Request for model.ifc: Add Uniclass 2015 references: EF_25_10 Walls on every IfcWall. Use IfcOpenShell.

First a look at what the model holds.

```python
import ifcopenshell

model = ifcopenshell.open("model.ifc")
print(model.schema)
print("classifications:", [c.Name for c in model.by_type("IfcClassification")])
for ifc_class in ("IfcDoor", "IfcRoof", "IfcStair", "IfcWall", "IfcWindow"):
    print(ifc_class, len(model.by_type(ifc_class)))
```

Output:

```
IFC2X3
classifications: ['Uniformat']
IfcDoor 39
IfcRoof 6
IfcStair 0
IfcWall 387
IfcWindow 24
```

```python
import ifcopenshell
import ifcopenshell.api.classification

model = ifcopenshell.open("model.ifc")

# IFC2X3 requires Source and Edition and has no link from the project to the system.
system = model.create_entity("IfcClassification", Source="NBS", Edition="2015", Name="Uniclass 2015")

codes = {
    "IfcWall": ("EF_25_10", "Walls"),
}
for ifc_class, (code, name) in codes.items():
    products = model.by_type(ifc_class)
    ifcopenshell.api.classification.add_reference(
        model, products=products, classification=system, identification=code, name=name
    )
    print(code, len(products))

model.write("model_updated.ifc")
```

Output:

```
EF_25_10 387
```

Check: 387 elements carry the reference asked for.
